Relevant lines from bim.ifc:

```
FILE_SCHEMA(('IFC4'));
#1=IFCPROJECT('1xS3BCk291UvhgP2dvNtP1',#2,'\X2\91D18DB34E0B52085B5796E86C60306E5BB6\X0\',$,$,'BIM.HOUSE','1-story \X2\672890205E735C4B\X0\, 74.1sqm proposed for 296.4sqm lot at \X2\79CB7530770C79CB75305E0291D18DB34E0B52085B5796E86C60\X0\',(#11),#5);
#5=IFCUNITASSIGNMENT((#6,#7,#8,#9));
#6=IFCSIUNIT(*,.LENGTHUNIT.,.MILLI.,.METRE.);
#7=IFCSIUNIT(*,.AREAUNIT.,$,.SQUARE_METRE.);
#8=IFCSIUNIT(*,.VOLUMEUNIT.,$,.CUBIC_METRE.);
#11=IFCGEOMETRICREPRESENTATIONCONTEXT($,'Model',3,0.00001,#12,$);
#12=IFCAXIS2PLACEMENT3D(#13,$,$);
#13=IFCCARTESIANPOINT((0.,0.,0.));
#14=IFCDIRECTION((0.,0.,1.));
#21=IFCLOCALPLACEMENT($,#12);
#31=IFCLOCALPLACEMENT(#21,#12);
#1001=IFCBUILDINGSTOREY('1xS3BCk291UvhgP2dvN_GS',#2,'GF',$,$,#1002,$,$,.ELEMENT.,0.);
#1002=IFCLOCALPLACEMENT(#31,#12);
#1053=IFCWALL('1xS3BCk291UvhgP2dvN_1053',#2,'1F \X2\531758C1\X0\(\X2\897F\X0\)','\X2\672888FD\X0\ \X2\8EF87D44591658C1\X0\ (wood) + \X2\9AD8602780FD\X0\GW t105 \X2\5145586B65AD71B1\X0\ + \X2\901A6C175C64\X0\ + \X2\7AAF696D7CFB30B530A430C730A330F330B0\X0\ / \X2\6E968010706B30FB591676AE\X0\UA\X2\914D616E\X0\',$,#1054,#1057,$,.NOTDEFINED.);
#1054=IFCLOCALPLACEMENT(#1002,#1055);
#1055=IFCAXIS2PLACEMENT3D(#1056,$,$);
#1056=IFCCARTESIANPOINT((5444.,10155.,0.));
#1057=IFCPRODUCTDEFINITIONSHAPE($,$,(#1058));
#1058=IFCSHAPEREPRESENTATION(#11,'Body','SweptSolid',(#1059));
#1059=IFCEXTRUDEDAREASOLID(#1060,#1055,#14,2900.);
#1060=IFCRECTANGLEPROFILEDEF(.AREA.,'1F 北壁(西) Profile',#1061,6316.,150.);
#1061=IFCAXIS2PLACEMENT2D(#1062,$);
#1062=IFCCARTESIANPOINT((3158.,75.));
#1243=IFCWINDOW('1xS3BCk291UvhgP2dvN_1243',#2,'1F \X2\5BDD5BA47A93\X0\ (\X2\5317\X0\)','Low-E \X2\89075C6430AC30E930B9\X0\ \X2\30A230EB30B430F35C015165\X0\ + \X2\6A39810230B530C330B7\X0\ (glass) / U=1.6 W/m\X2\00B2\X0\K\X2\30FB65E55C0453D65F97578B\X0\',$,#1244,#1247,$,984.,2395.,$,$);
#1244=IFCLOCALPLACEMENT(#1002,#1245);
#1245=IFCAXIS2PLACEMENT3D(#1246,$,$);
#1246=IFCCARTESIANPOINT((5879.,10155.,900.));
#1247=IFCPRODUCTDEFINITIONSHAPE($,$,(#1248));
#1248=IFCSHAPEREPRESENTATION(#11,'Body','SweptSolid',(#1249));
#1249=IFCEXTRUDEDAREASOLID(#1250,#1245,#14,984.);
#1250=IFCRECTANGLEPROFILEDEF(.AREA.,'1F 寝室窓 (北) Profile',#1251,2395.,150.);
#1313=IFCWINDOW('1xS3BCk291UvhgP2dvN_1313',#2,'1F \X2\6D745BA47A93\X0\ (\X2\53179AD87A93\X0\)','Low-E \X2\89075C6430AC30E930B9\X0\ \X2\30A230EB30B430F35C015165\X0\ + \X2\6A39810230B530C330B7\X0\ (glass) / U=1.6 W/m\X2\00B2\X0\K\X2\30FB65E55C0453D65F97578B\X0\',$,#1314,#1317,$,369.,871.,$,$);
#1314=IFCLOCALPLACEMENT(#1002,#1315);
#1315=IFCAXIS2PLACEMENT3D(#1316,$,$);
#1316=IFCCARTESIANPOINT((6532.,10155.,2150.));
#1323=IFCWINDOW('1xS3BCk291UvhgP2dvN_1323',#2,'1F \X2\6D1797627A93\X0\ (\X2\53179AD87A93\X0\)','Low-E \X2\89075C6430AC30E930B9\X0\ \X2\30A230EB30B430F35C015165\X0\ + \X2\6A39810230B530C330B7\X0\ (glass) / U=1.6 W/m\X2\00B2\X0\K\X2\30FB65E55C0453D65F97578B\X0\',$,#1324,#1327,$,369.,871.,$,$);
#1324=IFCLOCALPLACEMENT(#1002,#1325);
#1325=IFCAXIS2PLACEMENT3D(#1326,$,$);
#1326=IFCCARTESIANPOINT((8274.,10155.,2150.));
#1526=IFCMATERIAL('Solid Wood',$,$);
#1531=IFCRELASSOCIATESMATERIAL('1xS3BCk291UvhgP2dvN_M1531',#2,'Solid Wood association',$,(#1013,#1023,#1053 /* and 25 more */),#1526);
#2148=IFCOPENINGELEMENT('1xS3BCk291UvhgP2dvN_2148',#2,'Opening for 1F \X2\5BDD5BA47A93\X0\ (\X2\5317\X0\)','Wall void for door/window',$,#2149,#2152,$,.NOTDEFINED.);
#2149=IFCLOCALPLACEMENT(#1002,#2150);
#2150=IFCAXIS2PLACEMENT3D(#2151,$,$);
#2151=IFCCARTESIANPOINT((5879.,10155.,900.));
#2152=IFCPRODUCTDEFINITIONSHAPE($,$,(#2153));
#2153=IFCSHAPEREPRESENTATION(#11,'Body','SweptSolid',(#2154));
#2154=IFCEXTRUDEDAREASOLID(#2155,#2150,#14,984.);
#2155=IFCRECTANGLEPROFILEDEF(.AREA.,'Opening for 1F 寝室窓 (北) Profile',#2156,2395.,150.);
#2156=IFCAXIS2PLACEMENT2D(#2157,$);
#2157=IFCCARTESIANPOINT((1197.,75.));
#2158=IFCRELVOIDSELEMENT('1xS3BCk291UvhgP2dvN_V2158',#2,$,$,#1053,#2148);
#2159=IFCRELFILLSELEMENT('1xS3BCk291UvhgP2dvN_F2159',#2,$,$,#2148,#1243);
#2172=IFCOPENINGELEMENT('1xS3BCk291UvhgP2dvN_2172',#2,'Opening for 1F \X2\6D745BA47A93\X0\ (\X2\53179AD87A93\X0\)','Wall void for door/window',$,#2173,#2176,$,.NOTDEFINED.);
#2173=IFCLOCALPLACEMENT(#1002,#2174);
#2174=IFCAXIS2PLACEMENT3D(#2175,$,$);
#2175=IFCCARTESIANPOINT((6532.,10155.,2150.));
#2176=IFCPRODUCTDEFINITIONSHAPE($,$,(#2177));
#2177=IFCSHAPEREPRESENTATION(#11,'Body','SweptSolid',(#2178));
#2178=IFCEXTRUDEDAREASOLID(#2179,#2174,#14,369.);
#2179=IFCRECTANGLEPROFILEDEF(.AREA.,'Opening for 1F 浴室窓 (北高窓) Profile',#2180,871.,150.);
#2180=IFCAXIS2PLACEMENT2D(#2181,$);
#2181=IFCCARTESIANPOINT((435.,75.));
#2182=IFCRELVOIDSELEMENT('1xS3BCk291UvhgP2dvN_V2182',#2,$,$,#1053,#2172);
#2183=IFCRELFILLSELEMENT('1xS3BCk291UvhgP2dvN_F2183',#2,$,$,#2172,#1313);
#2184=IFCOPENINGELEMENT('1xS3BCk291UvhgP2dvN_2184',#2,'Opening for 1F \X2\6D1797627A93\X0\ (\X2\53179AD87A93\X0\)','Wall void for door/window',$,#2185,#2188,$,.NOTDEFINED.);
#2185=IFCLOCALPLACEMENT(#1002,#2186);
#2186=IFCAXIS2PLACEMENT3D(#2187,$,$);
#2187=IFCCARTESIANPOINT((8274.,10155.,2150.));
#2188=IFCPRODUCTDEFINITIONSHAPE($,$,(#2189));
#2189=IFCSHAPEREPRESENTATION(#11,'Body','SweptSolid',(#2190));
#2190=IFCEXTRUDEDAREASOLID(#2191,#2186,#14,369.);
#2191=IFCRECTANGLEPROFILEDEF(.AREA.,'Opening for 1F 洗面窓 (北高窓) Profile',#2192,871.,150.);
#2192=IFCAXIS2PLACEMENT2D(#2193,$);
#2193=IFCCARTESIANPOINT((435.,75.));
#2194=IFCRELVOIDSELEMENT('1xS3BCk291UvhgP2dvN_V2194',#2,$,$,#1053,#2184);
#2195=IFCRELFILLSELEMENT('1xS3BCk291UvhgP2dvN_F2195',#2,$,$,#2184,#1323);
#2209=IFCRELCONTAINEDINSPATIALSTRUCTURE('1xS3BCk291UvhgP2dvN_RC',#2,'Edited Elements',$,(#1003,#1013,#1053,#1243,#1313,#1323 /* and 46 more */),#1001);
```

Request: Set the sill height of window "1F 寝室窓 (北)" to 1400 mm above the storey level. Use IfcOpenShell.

```python
import numpy as np
import ifcopenshell
import ifcopenshell.api.geometry
import ifcopenshell.geom
import ifcopenshell.util.element
import ifcopenshell.util.placement
import ifcopenshell.util.shape
import ifcopenshell.util.unit

model = ifcopenshell.open("bim.ifc")
unit_scale = ifcopenshell.util.unit.calculate_unit_scale(model)

window = model.by_guid("1xS3BCk291UvhgP2dvN_1243")
opening = window.FillsVoids[0].RelatingOpeningElement
storey = ifcopenshell.util.element.get_container(window, ifc_class="IfcBuildingStorey")
level = ifcopenshell.util.placement.get_local_placement(storey.ObjectPlacement)[2, 3]

# The opening's origin need not be at the sill, so measure its lowest point.
shape = ifcopenshell.geom.create_shape(ifcopenshell.geom.settings(), opening)
bottom = ifcopenshell.util.shape.get_shape_bottom_elevation(shape, shape.geometry) / unit_scale
dz = level + 1.4 / unit_scale - bottom

shift = np.array([0.0, 0.0, dz])
# The window is not placed relative to its opening, so move both.
for product in (opening, window):
    matrix = ifcopenshell.util.placement.get_local_placement(product.ObjectPlacement)
    matrix[:3, 3] += shift
    ifcopenshell.api.geometry.edit_object_placement(model, product=product, matrix=matrix, is_si=False)

print(f"moved by {dz * unit_scale:+.3f} m")

model.write("bim_edited.ifc")
```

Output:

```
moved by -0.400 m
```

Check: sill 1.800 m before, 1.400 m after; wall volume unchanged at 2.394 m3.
